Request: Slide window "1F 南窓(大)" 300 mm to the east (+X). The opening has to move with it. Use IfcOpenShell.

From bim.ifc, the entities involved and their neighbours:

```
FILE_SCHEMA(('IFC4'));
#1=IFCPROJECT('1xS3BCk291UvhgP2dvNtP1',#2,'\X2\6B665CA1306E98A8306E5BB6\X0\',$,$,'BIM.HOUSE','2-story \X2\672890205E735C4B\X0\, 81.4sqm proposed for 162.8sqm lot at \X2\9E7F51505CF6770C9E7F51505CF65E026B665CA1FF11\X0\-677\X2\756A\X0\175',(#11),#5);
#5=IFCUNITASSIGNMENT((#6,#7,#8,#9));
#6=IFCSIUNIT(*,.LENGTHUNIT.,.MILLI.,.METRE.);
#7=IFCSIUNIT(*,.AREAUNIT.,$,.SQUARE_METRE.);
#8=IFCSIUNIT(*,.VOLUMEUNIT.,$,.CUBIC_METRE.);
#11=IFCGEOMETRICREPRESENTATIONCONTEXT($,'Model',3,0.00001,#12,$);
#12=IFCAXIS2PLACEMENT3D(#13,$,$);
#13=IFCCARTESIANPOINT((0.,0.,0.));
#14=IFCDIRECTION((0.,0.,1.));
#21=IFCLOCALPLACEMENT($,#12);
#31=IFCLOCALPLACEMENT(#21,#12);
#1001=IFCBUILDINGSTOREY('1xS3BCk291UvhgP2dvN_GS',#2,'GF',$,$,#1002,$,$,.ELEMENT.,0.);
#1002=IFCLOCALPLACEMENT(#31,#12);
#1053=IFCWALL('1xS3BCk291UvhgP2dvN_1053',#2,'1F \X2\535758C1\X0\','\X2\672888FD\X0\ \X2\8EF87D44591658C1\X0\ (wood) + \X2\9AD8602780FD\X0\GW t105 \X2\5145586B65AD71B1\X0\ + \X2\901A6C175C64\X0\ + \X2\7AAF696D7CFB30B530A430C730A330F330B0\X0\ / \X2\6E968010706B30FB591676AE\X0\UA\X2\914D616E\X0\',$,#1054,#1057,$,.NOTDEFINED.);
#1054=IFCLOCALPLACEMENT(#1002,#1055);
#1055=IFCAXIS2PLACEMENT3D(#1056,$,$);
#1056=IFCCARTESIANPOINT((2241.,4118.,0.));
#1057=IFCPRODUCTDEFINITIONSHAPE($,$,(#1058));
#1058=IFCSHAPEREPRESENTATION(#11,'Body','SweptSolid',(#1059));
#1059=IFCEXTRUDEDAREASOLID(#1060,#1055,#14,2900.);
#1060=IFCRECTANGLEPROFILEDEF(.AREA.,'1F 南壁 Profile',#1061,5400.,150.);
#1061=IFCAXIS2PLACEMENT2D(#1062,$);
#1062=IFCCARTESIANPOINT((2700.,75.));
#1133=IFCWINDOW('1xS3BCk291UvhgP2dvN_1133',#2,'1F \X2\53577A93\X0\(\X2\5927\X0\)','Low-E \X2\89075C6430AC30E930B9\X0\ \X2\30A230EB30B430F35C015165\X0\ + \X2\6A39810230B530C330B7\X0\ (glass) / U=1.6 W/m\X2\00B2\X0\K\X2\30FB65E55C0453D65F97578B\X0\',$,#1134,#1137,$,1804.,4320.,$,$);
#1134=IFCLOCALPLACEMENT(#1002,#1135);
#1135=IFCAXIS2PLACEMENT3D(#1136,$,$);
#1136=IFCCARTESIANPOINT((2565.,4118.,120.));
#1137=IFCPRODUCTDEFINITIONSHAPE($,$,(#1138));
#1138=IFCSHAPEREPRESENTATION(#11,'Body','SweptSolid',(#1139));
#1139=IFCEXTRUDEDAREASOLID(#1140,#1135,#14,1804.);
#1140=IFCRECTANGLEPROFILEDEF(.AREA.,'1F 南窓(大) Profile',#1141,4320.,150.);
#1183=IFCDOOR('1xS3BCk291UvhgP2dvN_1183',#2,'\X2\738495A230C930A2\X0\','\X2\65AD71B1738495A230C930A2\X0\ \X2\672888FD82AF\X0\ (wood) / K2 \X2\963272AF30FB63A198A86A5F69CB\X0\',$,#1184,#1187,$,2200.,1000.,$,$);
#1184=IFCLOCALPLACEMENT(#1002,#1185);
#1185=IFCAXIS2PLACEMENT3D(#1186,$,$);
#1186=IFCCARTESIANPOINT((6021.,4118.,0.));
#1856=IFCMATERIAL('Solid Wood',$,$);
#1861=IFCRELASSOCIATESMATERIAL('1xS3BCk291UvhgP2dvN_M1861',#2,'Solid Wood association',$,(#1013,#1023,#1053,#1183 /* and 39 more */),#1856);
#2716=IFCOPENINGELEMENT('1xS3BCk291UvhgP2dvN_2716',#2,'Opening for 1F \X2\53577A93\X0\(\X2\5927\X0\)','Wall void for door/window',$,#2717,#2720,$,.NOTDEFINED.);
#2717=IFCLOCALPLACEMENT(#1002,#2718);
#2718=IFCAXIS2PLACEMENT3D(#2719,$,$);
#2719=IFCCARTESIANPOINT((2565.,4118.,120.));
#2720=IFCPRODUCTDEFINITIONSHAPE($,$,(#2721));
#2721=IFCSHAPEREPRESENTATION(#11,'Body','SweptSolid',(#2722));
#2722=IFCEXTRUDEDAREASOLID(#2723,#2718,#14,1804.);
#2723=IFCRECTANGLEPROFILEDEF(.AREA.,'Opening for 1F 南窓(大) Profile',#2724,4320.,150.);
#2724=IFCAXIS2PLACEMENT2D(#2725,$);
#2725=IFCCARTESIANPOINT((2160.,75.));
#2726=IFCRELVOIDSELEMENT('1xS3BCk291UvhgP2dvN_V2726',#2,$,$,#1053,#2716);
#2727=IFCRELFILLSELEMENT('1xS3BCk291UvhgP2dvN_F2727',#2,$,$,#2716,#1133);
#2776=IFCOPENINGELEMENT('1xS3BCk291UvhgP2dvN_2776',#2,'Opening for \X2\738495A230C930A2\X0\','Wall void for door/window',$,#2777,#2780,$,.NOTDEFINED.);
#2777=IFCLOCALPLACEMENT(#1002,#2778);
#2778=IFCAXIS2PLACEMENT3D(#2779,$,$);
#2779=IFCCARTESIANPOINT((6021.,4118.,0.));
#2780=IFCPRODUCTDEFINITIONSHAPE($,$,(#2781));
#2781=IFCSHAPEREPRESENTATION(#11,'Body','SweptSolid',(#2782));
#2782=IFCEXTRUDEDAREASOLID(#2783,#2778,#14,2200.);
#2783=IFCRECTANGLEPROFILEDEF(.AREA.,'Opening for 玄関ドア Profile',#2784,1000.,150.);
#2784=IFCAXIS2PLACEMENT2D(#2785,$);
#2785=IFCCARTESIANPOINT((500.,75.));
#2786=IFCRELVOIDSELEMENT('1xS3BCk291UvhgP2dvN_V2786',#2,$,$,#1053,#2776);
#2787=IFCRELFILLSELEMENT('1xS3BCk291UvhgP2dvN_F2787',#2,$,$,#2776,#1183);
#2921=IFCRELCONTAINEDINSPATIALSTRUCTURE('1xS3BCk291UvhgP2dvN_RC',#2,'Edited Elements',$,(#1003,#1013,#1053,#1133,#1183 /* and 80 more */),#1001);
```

```python
import ifcopenshell
import ifcopenshell.api.geometry
import ifcopenshell.util.placement

model = ifcopenshell.open("bim.ifc")

window = model.by_guid("1xS3BCk291UvhgP2dvN_1133")
opening = window.FillsVoids[0].RelatingOpeningElement
wall = opening.VoidsElements[0].RelatingBuildingElement

wall_matrix = ifcopenshell.util.placement.get_local_placement(wall.ObjectPlacement)
shift = wall_matrix[:3, 0] * 300.0
before = ifcopenshell.util.placement.get_local_placement(window.ObjectPlacement)[:3, 3].copy()

# The window is not placed relative to its opening, so move both.
for product in (opening, window):
    matrix = ifcopenshell.util.placement.get_local_placement(product.ObjectPlacement)
    matrix[:3, 3] += shift
    ifcopenshell.api.geometry.edit_object_placement(model, product=product, matrix=matrix, is_si=False)

after = ifcopenshell.util.placement.get_local_placement(window.ObjectPlacement)[:3, 3]
print("window moved by", (after - before).round(3) + 0.0)

model.write("bim_rev.ifc")
```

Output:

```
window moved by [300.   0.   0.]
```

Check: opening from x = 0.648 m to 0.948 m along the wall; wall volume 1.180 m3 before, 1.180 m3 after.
